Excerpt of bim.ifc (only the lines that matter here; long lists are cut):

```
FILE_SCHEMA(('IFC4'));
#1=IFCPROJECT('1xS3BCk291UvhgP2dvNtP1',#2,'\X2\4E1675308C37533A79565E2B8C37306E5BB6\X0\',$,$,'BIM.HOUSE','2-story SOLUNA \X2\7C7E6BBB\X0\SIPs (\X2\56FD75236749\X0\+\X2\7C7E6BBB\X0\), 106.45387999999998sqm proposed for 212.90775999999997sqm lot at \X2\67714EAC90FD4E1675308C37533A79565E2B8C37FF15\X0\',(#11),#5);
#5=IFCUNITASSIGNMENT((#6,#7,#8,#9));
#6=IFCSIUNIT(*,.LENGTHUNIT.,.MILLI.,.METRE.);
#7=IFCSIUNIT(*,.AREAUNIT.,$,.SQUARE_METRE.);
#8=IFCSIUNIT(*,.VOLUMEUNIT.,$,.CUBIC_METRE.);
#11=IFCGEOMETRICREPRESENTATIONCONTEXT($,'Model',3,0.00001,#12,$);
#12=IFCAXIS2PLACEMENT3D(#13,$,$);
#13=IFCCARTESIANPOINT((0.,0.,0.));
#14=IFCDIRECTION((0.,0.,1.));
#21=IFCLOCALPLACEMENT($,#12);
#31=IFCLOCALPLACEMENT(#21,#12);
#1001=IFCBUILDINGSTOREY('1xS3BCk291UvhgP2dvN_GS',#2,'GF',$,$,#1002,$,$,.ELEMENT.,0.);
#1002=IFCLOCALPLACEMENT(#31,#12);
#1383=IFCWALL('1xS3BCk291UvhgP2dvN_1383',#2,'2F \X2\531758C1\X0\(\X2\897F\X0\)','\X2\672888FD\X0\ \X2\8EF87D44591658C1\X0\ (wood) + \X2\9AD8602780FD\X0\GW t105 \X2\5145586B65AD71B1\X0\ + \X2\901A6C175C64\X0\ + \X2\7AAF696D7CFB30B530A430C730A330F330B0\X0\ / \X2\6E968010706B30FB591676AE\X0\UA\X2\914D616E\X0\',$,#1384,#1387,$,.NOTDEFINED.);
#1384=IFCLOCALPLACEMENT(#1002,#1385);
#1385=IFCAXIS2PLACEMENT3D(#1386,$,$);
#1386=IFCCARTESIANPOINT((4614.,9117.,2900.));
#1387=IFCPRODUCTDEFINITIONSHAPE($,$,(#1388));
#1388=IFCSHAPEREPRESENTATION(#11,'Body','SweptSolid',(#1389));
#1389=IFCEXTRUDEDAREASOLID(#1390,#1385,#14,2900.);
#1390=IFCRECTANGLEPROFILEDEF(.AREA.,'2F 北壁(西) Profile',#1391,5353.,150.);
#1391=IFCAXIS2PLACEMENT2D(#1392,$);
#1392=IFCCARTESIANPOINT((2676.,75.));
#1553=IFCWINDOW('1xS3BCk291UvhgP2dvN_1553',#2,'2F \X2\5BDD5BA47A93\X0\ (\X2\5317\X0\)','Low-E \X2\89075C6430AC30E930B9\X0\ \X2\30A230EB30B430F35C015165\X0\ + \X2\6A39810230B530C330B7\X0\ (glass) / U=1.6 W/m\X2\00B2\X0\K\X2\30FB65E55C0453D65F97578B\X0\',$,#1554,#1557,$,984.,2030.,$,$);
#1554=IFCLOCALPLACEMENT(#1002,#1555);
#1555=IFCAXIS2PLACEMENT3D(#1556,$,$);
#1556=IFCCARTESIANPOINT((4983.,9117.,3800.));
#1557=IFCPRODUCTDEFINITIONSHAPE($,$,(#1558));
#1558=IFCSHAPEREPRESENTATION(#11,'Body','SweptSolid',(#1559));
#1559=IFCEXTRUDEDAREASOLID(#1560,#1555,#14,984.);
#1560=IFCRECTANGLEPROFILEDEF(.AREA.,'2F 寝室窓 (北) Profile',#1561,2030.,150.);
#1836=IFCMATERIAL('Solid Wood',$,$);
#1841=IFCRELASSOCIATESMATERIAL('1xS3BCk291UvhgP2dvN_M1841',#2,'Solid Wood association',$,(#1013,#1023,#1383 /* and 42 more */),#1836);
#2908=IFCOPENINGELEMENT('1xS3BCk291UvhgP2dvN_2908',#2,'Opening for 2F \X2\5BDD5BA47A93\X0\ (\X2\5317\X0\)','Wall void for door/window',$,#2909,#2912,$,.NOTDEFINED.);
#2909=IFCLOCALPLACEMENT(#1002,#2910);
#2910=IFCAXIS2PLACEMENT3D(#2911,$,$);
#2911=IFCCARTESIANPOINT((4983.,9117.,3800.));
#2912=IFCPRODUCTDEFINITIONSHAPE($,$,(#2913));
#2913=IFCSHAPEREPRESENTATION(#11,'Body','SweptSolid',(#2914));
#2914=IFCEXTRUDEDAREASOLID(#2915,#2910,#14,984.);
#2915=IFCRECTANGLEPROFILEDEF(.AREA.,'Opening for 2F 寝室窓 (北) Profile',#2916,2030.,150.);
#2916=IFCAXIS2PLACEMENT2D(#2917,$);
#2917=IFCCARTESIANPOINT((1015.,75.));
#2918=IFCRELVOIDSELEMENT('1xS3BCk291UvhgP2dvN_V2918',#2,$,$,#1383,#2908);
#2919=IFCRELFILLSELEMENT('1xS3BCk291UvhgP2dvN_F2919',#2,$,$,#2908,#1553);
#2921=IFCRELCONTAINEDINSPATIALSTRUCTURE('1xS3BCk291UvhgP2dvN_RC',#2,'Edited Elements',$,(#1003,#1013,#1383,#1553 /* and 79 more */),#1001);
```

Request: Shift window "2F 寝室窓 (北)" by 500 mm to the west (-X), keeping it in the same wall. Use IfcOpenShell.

```python
import ifcopenshell
import ifcopenshell.api.geometry
import ifcopenshell.util.placement

model = ifcopenshell.open("bim.ifc")

window = model.by_guid("1xS3BCk291UvhgP2dvN_1553")
opening = window.FillsVoids[0].RelatingOpeningElement
wall = opening.VoidsElements[0].RelatingBuildingElement

wall_matrix = ifcopenshell.util.placement.get_local_placement(wall.ObjectPlacement)
shift = wall_matrix[:3, 0] * -500.0
before = ifcopenshell.util.placement.get_local_placement(window.ObjectPlacement)[:3, 3].copy()

# The window is not placed relative to its opening, so move both.
for product in (opening, window):
    matrix = ifcopenshell.util.placement.get_local_placement(product.ObjectPlacement)
    matrix[:3, 3] += shift
    ifcopenshell.api.geometry.edit_object_placement(model, product=product, matrix=matrix, is_si=False)

after = ifcopenshell.util.placement.get_local_placement(window.ObjectPlacement)[:3, 3]
print("window moved by", (after - before).round(3) + 0.0)

model.write("bim_v2.ifc")
```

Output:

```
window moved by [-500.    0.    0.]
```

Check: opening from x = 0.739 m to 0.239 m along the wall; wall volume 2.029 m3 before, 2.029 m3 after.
